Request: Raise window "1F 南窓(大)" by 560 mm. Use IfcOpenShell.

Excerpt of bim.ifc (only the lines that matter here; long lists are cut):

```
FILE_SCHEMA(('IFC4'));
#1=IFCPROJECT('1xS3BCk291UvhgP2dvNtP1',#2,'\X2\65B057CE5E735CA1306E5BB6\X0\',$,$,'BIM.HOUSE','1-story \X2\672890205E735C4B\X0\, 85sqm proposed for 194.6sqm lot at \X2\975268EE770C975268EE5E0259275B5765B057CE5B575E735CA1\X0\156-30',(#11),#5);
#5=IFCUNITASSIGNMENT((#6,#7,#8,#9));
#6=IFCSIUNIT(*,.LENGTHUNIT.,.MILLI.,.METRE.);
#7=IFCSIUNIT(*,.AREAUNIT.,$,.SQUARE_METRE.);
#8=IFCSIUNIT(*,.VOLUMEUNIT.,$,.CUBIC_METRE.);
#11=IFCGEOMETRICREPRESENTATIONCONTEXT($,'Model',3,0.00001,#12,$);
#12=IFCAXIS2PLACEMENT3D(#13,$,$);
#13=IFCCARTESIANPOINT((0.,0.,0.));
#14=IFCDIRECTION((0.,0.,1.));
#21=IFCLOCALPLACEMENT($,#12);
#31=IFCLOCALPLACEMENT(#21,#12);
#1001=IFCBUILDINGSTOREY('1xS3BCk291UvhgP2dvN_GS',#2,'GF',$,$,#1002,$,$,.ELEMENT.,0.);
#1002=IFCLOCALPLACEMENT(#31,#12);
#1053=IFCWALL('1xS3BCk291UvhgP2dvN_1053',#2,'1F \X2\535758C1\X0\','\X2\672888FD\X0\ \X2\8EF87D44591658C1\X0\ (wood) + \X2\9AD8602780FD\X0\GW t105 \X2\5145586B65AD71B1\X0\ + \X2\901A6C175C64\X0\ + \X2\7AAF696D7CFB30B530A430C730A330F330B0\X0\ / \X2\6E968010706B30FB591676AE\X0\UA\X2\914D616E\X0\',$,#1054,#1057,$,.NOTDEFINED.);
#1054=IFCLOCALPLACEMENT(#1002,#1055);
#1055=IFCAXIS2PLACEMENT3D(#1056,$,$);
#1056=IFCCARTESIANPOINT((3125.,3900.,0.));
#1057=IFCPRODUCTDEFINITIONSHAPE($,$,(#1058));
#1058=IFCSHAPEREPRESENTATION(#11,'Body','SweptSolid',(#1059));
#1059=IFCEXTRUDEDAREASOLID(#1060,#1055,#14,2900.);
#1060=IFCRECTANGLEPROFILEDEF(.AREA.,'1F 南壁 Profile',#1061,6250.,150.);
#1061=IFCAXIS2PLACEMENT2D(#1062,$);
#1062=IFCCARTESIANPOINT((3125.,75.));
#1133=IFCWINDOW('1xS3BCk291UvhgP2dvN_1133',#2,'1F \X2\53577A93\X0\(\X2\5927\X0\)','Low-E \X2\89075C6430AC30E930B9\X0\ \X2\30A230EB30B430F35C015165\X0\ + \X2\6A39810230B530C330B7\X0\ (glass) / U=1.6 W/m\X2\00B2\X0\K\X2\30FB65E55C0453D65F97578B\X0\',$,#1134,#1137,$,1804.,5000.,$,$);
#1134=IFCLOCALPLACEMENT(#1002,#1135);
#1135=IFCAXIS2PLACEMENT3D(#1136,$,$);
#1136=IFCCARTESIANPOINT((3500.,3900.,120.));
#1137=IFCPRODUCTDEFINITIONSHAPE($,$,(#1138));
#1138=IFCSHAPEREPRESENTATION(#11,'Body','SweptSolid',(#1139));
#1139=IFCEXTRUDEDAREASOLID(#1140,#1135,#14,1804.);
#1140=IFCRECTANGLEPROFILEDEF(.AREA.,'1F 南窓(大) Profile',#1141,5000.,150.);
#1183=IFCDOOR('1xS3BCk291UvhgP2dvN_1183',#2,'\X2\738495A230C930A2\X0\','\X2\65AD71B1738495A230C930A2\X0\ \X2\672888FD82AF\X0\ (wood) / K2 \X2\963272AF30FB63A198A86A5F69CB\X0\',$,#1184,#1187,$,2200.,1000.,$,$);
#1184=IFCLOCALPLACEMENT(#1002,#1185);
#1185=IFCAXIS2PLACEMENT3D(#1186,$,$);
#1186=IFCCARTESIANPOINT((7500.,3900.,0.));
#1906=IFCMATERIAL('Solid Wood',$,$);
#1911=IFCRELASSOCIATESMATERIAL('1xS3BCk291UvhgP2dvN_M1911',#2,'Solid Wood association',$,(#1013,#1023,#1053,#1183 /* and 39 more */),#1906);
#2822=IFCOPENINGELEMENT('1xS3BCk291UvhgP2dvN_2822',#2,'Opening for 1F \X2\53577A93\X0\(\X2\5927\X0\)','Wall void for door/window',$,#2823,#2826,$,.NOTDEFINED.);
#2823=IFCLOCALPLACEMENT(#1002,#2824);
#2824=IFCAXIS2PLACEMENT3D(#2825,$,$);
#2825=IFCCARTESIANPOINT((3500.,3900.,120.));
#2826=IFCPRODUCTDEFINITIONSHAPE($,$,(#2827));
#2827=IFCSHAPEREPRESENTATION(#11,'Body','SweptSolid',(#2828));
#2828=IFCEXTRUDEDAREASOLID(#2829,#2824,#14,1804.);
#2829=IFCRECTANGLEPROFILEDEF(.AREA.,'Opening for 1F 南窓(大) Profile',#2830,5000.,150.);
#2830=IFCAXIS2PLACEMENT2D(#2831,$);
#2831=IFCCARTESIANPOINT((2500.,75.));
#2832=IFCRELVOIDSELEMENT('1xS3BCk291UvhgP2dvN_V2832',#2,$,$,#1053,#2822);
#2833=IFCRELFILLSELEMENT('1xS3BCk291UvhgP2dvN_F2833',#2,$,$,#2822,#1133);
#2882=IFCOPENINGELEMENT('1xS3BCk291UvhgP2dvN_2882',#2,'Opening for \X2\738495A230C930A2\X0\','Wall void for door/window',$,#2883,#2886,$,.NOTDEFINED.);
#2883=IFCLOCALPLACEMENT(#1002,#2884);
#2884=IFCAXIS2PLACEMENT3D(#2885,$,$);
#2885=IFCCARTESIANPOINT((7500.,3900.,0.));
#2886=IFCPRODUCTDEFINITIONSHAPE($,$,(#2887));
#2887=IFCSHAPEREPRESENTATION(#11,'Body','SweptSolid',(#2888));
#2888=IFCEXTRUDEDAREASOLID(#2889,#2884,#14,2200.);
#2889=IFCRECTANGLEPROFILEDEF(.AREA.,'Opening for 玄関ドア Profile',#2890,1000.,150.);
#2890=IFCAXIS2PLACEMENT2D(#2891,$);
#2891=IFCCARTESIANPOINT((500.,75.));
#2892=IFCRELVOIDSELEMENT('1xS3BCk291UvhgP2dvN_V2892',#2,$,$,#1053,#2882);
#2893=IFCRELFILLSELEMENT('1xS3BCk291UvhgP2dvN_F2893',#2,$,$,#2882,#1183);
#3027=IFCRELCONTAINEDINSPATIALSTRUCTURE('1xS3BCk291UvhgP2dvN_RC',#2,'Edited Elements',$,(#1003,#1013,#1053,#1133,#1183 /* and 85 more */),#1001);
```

```python
import numpy as np
import ifcopenshell
import ifcopenshell.api.geometry
import ifcopenshell.util.placement
import ifcopenshell.util.unit

model = ifcopenshell.open("bim.ifc")
unit_scale = ifcopenshell.util.unit.calculate_unit_scale(model)

window = model.by_id(1133)
opening = window.FillsVoids[0].RelatingOpeningElement
dz = 0.56 / unit_scale

shift = np.array([0.0, 0.0, dz])
# The window is not placed relative to its opening, so move both.
for product in (opening, window):
    matrix = ifcopenshell.util.placement.get_local_placement(product.ObjectPlacement)
    matrix[:3, 3] += shift
    ifcopenshell.api.geometry.edit_object_placement(model, product=product, matrix=matrix, is_si=False)

print(f"moved by {dz * unit_scale:+.3f} m")

model.write("bim_updated.ifc")
```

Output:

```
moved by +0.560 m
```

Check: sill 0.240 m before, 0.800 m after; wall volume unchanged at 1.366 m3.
